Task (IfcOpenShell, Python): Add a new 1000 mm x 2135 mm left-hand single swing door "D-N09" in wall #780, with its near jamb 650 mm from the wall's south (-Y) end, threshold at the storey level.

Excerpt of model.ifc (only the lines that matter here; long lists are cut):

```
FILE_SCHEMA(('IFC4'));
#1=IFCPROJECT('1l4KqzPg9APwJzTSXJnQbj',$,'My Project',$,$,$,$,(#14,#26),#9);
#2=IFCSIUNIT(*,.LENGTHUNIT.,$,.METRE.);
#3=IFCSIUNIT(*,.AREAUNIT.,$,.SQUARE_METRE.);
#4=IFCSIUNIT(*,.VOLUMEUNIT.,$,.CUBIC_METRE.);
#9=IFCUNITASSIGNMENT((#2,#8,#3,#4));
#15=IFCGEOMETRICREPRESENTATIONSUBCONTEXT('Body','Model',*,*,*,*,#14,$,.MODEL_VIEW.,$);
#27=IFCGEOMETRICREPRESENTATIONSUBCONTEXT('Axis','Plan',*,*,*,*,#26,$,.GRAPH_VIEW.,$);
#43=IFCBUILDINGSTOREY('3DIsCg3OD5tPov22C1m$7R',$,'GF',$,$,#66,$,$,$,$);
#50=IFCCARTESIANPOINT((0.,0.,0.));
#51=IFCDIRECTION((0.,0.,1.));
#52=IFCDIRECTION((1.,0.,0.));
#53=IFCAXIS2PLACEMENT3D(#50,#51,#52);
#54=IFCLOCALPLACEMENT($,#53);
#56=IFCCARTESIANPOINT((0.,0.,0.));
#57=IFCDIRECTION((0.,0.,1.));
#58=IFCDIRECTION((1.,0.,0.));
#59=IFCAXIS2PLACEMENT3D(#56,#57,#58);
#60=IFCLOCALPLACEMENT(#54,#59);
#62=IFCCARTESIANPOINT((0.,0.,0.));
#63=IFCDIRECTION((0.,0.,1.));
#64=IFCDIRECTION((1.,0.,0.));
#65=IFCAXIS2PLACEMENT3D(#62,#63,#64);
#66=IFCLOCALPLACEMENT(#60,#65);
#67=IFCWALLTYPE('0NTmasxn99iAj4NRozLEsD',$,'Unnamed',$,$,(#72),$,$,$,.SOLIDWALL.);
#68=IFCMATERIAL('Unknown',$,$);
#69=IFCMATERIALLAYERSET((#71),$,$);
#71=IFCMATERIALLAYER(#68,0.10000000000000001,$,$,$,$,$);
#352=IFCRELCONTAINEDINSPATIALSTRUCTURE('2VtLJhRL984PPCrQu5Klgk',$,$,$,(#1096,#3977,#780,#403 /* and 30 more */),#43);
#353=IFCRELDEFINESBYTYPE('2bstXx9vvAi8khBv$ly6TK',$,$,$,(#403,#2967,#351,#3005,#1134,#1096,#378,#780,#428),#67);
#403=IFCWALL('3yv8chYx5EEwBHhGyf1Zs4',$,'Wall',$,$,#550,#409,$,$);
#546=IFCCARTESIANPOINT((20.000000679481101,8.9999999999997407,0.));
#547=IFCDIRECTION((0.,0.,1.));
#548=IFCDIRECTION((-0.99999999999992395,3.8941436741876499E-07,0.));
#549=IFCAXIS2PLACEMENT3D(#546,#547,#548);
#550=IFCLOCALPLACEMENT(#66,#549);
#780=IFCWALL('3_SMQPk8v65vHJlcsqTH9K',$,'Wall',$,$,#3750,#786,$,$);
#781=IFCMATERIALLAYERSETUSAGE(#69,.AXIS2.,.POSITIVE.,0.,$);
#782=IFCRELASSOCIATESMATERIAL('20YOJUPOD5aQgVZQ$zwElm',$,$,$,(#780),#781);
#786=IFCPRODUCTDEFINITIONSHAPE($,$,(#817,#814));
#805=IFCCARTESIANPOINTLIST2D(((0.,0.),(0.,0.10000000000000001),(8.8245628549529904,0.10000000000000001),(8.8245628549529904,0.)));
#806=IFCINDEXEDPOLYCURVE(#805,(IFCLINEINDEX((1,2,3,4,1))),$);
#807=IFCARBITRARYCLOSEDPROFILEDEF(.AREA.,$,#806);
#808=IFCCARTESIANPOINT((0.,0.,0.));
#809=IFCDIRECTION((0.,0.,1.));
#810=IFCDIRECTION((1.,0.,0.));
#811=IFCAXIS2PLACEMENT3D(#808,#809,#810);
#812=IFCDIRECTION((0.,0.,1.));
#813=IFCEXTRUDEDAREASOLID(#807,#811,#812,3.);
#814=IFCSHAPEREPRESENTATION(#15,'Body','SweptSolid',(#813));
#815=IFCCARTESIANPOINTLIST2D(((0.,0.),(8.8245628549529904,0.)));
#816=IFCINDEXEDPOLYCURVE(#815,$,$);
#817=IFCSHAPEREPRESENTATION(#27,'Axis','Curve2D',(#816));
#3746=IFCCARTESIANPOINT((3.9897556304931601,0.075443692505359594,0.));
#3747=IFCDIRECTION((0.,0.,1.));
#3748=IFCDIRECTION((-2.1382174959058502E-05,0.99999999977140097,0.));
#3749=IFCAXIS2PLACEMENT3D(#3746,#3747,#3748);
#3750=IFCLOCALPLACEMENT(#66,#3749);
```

```python
import numpy as np
import ifcopenshell
import ifcopenshell.api.feature
import ifcopenshell.api.geometry
import ifcopenshell.api.root
import ifcopenshell.api.spatial
import ifcopenshell.geom
import ifcopenshell.util.element
import ifcopenshell.util.placement
import ifcopenshell.util.representation
import ifcopenshell.util.shape
import ifcopenshell.util.unit

model = ifcopenshell.open("model.ifc")
unit_scale = ifcopenshell.util.unit.calculate_unit_scale(model)
settings = ifcopenshell.geom.settings()


def volume(element):
    """Net volume in cubic metres, openings subtracted."""
    shape = ifcopenshell.geom.create_shape(settings, element)
    return ifcopenshell.util.shape.get_volume(shape.geometry)


wall = model.by_guid("3_SMQPk8v65vHJlcsqTH9K")
storey = ifcopenshell.util.element.get_container(wall, ifc_class="IfcBuildingStorey")
context = ifcopenshell.util.representation.get_context(model, "Model", "Body", "MODEL_VIEW")
before = volume(wall)

width, height, from_end, sill = 1, 2.135, 0.65, 0.0  # metres

# The wall runs along its own X axis, and the end named is its -X end.
wall_shape = ifcopenshell.geom.create_shape(settings, wall)
x, y, z = ifcopenshell.util.shape.get_vertices(wall_shape.geometry).T
start = x.min() + from_end
face, thickness = float(y.min()), float(y.max() - y.min())
wall_matrix = ifcopenshell.util.placement.get_local_placement(wall.ObjectPlacement)
level = ifcopenshell.util.placement.get_local_placement(storey.ObjectPlacement)[2, 3]


def in_wall(x, y):
    """Placement at x, y metres in the wall's axes, at sill height."""
    matrix = wall_matrix.copy()
    matrix[:, 3] = wall_matrix @ np.array([x / unit_scale, y / unit_scale, 0.0, 1.0])
    matrix[2, 3] = level + sill / unit_scale
    return matrix


# Opening: a box that overshoots both wall faces by 50 mm.
opening = ifcopenshell.api.root.create_entity(model, ifc_class="IfcOpeningElement", predefined_type="OPENING")
box = ifcopenshell.api.geometry.add_wall_representation(
    model, context=context, length=width, height=height, thickness=thickness + 0.1
)
ifcopenshell.api.geometry.assign_representation(model, product=opening, representation=box)
ifcopenshell.api.geometry.edit_object_placement(model, product=opening, matrix=in_wall(start, face - 0.05), is_si=False)
ifcopenshell.api.feature.add_feature(model, feature=opening, element=wall)

door = ifcopenshell.api.root.create_entity(model, ifc_class="IfcDoor", name="D-N09", predefined_type="DOOR")
door.OverallWidth, door.OverallHeight = width / unit_scale, height / unit_scale
door.OperationType = "SINGLE_SWING_LEFT"
body = ifcopenshell.api.geometry.add_door_representation(
    model,
    context=context,
    overall_width=door.OverallWidth,
    overall_height=door.OverallHeight,
    operation_type="SINGLE_SWING_LEFT",
    lining_properties={"LiningDepth": thickness / unit_scale, "ThresholdDepth": thickness / unit_scale},
)
ifcopenshell.api.geometry.assign_representation(model, product=door, representation=body)
ifcopenshell.api.spatial.assign_container(model, products=[door], relating_structure=storey)
ifcopenshell.api.feature.add_filling(model, opening=opening, element=door)

# The lining spans the wall, so the door starts at the wall face.
ifcopenshell.api.geometry.edit_object_placement(model, product=door, matrix=in_wall(start, face), is_si=False)

after = volume(wall)

print(f"wall volume {before:.3f} -> {after:.3f} m3")

model.write("model_v2.ifc")
```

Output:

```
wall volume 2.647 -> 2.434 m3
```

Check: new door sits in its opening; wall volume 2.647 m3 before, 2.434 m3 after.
